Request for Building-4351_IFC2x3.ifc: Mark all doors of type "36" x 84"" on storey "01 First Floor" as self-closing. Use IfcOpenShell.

First a look at what the model holds.

```python
import ifcopenshell
import ifcopenshell.util.element

model = ifcopenshell.open("Building-4351_IFC2x3.ifc")
print(model.schema)
storey = next(s for s in model.by_type("IfcBuildingStorey") if s.Name == "01 First Floor")
doors = [e for e in ifcopenshell.util.element.get_decomposition(storey) if e.is_a("IfcDoor")]
seen = {}
for e in doors:
    element_type = ifcopenshell.util.element.get_type(e)
    key = (element_type.Name if element_type != e and element_type else None, ifcopenshell.util.element.get_pset(e, "Pset_DoorCommon", "SelfClosing"))
    seen[key] = seen.get(key, 0) + 1
for (name, value), count in sorted(seen.items(), key=str):
    print(count, "x", name, "|", value)
```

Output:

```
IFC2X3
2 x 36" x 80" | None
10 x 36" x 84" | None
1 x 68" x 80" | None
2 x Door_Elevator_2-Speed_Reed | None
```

```python
import ifcopenshell
import ifcopenshell.api.pset
import ifcopenshell.util.element

model = ifcopenshell.open("Building-4351_IFC2x3.ifc")

storey = next(s for s in model.by_type("IfcBuildingStorey") if s.Name == "01 First Floor")
doors = [e for e in ifcopenshell.util.element.get_decomposition(storey) if e.is_a("IfcDoor")]

count = 0
for e in doors:
    element_type = ifcopenshell.util.element.get_type(e)
    if element_type in (None, e) or element_type.Name != '36" x 84"':
        continue
    # add_pset returns the element's existing set when there is one.
    pset = ifcopenshell.api.pset.add_pset(model, product=e, name="Pset_DoorCommon")
    ifcopenshell.api.pset.edit_pset(model, pset=pset, properties={"SelfClosing": True})
    count += 1

print(count, "doors updated")

model.write("Building-4351_IFC2x3_v2.ifc")
```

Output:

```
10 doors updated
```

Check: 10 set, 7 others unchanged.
